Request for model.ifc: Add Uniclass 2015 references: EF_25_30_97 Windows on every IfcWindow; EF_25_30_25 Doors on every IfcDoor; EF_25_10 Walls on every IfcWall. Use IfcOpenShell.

First a look at what the model holds.

```python
import ifcopenshell

model = ifcopenshell.open("model.ifc")
print(model.schema)
print("classifications:", [c.Name for c in model.by_type("IfcClassification")])
for ifc_class in ("IfcDoor", "IfcRoof", "IfcStair", "IfcWall", "IfcWindow"):
    print(ifc_class, len(model.by_type(ifc_class)))
```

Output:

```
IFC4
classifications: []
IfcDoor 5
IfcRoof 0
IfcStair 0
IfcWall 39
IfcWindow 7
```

```python
import ifcopenshell
import ifcopenshell.api.classification

model = ifcopenshell.open("model.ifc")

system = ifcopenshell.api.classification.add_classification(model, classification="Uniclass 2015")

codes = {
    "IfcWindow": ("EF_25_30_97", "Windows"),
    "IfcDoor": ("EF_25_30_25", "Doors"),
    "IfcWall": ("EF_25_10", "Walls"),
}
for ifc_class, (code, name) in codes.items():
    products = model.by_type(ifc_class)
    ifcopenshell.api.classification.add_reference(
        model, products=products, classification=system, identification=code, name=name
    )
    print(code, len(products))

model.write("model_v2.ifc")
```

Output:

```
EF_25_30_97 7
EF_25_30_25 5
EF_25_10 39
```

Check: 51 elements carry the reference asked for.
